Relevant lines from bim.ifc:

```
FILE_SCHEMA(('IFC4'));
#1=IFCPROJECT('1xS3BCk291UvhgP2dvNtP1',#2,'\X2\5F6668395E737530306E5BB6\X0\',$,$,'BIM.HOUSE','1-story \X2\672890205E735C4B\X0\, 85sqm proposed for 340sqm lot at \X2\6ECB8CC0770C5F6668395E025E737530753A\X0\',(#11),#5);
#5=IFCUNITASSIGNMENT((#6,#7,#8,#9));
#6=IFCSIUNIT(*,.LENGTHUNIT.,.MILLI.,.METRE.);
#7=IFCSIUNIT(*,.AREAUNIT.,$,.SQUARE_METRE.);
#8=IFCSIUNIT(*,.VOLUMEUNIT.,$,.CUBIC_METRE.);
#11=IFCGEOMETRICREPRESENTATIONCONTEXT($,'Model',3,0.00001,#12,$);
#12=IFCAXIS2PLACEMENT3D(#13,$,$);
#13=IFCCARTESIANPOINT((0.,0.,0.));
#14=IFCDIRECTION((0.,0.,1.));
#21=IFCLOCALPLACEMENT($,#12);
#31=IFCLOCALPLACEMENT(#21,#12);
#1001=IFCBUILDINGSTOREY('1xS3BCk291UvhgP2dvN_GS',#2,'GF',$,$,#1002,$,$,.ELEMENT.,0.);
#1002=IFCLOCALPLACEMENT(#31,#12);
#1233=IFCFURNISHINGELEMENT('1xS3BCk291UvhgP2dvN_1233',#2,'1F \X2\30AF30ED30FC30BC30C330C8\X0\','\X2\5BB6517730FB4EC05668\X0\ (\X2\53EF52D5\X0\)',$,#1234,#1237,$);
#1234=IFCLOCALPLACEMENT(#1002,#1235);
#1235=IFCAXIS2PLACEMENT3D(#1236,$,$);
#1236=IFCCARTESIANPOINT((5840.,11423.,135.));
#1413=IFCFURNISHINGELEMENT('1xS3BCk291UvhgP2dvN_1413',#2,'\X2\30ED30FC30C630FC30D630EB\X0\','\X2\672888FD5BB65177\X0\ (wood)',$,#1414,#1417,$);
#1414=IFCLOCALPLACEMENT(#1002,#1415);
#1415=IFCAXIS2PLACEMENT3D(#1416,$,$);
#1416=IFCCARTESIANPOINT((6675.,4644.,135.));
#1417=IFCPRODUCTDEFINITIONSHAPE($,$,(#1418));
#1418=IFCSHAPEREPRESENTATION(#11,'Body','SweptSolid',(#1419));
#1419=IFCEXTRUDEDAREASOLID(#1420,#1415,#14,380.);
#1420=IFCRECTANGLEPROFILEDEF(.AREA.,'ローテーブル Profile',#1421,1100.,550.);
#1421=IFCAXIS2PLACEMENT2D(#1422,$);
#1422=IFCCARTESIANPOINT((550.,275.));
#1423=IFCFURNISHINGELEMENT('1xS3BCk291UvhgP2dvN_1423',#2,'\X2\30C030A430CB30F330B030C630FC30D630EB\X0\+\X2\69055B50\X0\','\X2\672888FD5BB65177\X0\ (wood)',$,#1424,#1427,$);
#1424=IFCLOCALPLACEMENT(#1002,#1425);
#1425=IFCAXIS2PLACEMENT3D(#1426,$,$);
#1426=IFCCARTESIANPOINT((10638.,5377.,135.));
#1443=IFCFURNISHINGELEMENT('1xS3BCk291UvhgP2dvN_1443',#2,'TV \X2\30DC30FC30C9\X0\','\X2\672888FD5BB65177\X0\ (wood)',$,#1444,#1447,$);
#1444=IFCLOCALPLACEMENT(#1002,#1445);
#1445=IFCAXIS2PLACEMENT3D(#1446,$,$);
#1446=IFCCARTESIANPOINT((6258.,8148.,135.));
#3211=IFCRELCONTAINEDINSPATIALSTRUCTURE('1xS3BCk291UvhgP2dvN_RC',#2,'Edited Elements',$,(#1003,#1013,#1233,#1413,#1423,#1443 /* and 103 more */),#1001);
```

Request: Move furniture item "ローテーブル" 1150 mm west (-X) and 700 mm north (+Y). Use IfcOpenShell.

```python
import ifcopenshell
import ifcopenshell.api.geometry
import ifcopenshell.util.placement

model = ifcopenshell.open("bim.ifc")

item = model.by_guid("1xS3BCk291UvhgP2dvN_1413")
matrix = ifcopenshell.util.placement.get_local_placement(item.ObjectPlacement)
matrix[0, 3] -= 1150.0
matrix[1, 3] += 700.0
ifcopenshell.api.geometry.edit_object_placement(model, product=item, matrix=matrix, is_si=False)

print(ifcopenshell.util.placement.get_local_placement(item.ObjectPlacement).round(3) + 0.0)

model.write("bim-out.ifc")
```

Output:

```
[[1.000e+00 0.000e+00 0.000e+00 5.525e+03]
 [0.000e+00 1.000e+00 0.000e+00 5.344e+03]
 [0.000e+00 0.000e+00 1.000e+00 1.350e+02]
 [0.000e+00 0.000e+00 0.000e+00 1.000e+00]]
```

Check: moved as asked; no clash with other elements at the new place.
